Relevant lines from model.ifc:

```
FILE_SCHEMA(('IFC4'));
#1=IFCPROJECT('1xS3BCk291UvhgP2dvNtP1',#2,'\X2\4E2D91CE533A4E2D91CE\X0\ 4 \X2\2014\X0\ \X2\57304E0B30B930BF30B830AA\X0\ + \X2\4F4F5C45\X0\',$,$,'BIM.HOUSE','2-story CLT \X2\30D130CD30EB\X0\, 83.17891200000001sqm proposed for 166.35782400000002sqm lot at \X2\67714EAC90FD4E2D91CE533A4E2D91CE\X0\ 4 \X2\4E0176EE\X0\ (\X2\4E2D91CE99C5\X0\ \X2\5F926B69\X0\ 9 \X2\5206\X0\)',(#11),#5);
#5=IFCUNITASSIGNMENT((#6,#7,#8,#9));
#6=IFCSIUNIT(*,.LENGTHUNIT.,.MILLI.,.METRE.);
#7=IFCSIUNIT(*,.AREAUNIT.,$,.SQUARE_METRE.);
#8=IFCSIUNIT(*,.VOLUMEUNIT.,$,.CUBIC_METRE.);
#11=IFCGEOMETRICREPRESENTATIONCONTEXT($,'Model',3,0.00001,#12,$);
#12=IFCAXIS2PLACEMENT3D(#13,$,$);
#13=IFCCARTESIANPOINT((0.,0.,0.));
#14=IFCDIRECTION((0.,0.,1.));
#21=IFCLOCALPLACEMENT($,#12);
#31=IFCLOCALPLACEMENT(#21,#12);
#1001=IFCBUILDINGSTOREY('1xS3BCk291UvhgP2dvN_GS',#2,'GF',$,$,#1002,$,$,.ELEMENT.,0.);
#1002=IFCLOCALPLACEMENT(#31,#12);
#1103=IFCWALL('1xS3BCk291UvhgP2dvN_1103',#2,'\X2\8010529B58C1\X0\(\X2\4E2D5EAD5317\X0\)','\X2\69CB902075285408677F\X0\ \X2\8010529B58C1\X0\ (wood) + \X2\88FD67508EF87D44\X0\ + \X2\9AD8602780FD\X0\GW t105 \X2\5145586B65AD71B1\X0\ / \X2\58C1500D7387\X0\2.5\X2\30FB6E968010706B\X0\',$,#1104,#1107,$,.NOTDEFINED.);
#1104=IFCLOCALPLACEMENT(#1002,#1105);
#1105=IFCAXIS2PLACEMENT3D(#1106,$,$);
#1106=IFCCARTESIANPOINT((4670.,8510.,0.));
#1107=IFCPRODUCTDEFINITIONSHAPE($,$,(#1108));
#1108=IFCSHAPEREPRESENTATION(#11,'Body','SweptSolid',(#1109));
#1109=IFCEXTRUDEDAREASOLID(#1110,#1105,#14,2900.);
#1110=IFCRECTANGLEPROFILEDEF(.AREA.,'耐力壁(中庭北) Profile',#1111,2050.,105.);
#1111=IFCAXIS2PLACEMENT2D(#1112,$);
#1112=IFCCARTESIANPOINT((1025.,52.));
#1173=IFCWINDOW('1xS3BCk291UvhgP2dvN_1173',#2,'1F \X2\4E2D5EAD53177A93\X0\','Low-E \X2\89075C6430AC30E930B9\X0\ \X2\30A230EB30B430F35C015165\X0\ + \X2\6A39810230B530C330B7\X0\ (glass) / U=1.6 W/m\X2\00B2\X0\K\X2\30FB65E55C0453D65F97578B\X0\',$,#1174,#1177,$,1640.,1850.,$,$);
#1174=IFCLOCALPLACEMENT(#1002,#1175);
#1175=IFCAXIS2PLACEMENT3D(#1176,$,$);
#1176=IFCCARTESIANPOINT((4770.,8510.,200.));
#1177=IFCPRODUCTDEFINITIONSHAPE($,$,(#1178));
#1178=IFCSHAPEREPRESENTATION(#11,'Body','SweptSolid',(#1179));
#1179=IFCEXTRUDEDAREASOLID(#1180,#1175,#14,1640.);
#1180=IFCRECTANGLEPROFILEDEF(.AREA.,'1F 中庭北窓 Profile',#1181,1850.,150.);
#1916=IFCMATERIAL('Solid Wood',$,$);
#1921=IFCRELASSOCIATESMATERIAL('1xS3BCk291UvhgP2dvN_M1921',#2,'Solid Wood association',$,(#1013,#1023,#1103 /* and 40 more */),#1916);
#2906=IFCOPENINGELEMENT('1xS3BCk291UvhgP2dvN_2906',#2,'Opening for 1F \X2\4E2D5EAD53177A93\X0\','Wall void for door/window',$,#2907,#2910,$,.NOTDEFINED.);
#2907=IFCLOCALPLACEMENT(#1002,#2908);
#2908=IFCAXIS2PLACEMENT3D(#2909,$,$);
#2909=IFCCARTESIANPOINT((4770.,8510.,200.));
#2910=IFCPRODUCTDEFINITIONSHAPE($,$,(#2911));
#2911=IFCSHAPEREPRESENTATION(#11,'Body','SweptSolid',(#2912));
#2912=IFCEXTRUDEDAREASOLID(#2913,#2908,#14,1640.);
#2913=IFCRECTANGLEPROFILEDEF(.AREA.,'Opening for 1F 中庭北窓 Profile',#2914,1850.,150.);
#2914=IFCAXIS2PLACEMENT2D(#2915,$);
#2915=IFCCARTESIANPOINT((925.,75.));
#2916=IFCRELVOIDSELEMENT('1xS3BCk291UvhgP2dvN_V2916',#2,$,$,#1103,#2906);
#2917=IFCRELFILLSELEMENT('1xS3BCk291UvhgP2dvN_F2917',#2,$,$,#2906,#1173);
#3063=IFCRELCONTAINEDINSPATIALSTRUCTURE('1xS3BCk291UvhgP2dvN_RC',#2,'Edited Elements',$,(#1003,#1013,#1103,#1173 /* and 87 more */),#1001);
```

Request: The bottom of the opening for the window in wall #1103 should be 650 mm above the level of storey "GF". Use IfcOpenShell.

```python
import numpy as np
import ifcopenshell
import ifcopenshell.api.geometry
import ifcopenshell.geom
import ifcopenshell.util.element
import ifcopenshell.util.placement
import ifcopenshell.util.shape
import ifcopenshell.util.unit

model = ifcopenshell.open("model.ifc")
unit_scale = ifcopenshell.util.unit.calculate_unit_scale(model)

window = model.by_guid("1xS3BCk291UvhgP2dvN_1173")
opening = window.FillsVoids[0].RelatingOpeningElement
storey = ifcopenshell.util.element.get_container(window, ifc_class="IfcBuildingStorey")
level = ifcopenshell.util.placement.get_local_placement(storey.ObjectPlacement)[2, 3]

# The opening's origin need not be at the sill, so measure its lowest point.
shape = ifcopenshell.geom.create_shape(ifcopenshell.geom.settings(), opening)
bottom = ifcopenshell.util.shape.get_shape_bottom_elevation(shape, shape.geometry) / unit_scale
dz = level + 0.65 / unit_scale - bottom

shift = np.array([0.0, 0.0, dz])
# The window is not placed relative to its opening, so move both.
for product in (opening, window):
    matrix = ifcopenshell.util.placement.get_local_placement(product.ObjectPlacement)
    matrix[:3, 3] += shift
    ifcopenshell.api.geometry.edit_object_placement(model, product=product, matrix=matrix, is_si=False)

print(f"moved by {dz * unit_scale:+.3f} m")

model.write("model_updated.ifc")
```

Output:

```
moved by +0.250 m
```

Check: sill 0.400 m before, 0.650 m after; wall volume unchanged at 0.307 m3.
